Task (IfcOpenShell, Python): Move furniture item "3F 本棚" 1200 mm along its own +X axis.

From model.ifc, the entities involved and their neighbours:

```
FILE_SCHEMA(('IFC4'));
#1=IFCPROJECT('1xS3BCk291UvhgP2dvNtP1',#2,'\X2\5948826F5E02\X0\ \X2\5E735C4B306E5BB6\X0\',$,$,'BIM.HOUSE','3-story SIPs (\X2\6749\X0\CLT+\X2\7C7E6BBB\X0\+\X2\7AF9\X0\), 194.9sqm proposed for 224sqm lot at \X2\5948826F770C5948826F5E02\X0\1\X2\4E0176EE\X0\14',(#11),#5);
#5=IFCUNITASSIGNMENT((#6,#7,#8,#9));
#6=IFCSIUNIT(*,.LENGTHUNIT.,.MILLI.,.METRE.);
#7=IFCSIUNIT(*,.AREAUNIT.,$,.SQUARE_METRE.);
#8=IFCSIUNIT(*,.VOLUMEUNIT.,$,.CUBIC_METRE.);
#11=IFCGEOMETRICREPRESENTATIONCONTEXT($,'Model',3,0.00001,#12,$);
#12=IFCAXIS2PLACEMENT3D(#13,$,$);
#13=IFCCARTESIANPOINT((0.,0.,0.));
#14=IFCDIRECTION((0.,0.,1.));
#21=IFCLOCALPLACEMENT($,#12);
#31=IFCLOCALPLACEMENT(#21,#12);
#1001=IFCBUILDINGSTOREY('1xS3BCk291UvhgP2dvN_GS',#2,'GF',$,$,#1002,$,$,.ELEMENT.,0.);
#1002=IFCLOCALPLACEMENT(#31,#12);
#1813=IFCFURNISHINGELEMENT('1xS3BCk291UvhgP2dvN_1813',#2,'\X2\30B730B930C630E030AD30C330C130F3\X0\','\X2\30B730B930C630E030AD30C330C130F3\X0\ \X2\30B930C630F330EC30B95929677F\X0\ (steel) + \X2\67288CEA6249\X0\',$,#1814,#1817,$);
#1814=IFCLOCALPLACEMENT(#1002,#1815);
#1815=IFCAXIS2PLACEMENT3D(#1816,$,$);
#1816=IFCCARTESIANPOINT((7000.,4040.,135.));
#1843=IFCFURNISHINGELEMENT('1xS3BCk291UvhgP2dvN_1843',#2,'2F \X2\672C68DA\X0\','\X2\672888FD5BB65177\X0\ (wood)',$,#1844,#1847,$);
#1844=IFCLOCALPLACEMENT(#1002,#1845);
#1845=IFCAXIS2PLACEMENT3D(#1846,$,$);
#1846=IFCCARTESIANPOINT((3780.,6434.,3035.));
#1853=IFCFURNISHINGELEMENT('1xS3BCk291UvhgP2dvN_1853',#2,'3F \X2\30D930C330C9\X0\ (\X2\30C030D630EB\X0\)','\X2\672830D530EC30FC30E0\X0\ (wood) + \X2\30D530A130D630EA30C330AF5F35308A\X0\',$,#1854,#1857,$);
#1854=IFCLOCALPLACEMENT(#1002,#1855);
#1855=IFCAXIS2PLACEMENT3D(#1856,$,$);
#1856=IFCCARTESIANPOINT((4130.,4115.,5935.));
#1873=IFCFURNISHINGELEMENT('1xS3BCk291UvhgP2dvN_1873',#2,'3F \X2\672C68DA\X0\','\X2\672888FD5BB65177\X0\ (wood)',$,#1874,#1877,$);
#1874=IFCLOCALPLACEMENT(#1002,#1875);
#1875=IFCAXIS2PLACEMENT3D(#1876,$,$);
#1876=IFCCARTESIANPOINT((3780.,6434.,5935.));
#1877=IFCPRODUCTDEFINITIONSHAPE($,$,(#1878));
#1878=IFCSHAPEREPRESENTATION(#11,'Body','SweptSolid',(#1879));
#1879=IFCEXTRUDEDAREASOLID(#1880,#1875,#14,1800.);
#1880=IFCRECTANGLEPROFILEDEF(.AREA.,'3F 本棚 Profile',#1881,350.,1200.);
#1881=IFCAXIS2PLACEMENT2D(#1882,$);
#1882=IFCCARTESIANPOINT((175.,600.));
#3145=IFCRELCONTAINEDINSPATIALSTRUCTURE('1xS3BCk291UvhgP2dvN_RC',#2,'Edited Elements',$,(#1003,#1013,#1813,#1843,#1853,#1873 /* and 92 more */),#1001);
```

```python
import ifcopenshell
import ifcopenshell.api.geometry
import ifcopenshell.util.placement
import ifcopenshell.util.unit

model = ifcopenshell.open("model.ifc")
unit_scale = ifcopenshell.util.unit.calculate_unit_scale(model)

item = model.by_guid("1xS3BCk291UvhgP2dvN_1873")
matrix = ifcopenshell.util.placement.get_local_placement(item.ObjectPlacement)
matrix[:3, 3] += matrix[:3, 0] * 1.2 / unit_scale
ifcopenshell.api.geometry.edit_object_placement(model, product=item, matrix=matrix, is_si=False)

print(ifcopenshell.util.placement.get_local_placement(item.ObjectPlacement).round(3) + 0.0)

model.write("model_rev.ifc")
```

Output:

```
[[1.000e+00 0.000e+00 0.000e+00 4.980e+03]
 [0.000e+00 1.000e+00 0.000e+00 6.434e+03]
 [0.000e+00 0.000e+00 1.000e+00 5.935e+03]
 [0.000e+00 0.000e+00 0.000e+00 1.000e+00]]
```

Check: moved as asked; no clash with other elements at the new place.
